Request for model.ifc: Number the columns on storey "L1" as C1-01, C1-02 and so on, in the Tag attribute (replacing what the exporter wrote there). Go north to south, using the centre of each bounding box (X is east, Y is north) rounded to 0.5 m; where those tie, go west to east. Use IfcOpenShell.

First a look at what the model holds.

```python
import ifcopenshell
import ifcopenshell.util.element
import ifcopenshell.util.placement

model = ifcopenshell.open("model.ifc")
print(model.schema)
storey = next(s for s in model.by_type("IfcBuildingStorey") if s.Name == "L1")
columns = [e for e in ifcopenshell.util.element.get_decomposition(storey) if e.is_a("IfcColumn")]
for e in sorted(columns, key=lambda e: e.id()):
    origin = ifcopenshell.util.placement.get_local_placement(e.ObjectPlacement)[:3, 3]
    print(e.id(), e.Tag, e.Name, origin.round(2) + 0.0, sep=" | ")
```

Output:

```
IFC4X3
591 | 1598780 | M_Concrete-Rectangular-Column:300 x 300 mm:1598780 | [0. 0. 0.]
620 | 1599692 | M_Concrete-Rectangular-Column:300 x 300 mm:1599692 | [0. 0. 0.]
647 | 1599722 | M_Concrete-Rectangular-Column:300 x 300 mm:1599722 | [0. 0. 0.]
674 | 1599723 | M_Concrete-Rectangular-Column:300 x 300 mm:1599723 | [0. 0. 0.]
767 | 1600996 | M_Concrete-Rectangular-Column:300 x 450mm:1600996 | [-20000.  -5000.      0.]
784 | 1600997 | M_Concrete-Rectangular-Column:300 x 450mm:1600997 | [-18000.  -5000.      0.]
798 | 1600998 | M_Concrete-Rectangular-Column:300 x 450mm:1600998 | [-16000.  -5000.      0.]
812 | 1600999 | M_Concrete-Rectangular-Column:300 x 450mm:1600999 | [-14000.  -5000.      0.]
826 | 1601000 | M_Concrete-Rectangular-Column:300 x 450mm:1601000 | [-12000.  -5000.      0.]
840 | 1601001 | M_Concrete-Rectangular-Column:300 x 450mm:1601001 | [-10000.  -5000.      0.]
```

```python
import ifcopenshell
import ifcopenshell.geom
import ifcopenshell.util.element
import ifcopenshell.util.shape

model = ifcopenshell.open("model.ifc")
settings = ifcopenshell.geom.settings()
settings.set("use-world-coords", True)


def centre(element):
    shape = ifcopenshell.geom.create_shape(settings, element)
    return ifcopenshell.util.shape.get_bbox_centroid(shape.geometry)


storey = next(s for s in model.by_type("IfcBuildingStorey") if s.Name == "L1")
columns = [e for e in ifcopenshell.util.element.get_decomposition(storey) if e.is_a("IfcColumn")]

# Insertion points can sit at a corner or the storey origin, so sort by the geometry (in metres).
centres = {e: centre(e) for e in columns}
columns.sort(key=lambda e: (-round(centres[e][1] / 0.5), centres[e][0]))

for i, e in enumerate(columns, start=1):
    number = f"C1-{i:02d}"
    e.Tag = number
    print(e.id(), number)

model.write("model_rev.ifc")
```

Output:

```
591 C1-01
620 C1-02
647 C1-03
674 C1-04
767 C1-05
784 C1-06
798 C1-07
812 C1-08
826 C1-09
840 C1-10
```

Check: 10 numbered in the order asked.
